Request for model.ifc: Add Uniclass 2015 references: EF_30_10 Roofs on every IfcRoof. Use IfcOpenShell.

First a look at what the model holds.

```python
import ifcopenshell

model = ifcopenshell.open("model.ifc")
print(model.schema)
print("classifications:", [c.Name for c in model.by_type("IfcClassification")])
for ifc_class in ("IfcDoor", "IfcRoof", "IfcStair", "IfcWall", "IfcWindow"):
    print(ifc_class, len(model.by_type(ifc_class)))
```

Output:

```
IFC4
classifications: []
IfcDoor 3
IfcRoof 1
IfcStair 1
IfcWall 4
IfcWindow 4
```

```python
import ifcopenshell
import ifcopenshell.api.classification

model = ifcopenshell.open("model.ifc")

system = ifcopenshell.api.classification.add_classification(model, classification="Uniclass 2015")

codes = {
    "IfcRoof": ("EF_30_10", "Roofs"),
}
for ifc_class, (code, name) in codes.items():
    products = model.by_type(ifc_class)
    ifcopenshell.api.classification.add_reference(
        model, products=products, classification=system, identification=code, name=name
    )
    print(code, len(products))

model.write("model_rev.ifc")
```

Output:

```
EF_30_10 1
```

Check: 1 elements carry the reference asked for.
